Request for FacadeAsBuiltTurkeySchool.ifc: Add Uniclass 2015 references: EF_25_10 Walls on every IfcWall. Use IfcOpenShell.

First a look at what the model holds.

```python
import ifcopenshell

model = ifcopenshell.open("FacadeAsBuiltTurkeySchool.ifc")
print(model.schema)
print("classifications:", [c.Name for c in model.by_type("IfcClassification")])
for ifc_class in ("IfcDoor", "IfcRoof", "IfcStair", "IfcWall", "IfcWindow"):
    print(ifc_class, len(model.by_type(ifc_class)))
```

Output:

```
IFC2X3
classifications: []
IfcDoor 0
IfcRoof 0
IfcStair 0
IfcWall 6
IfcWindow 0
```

```python
import ifcopenshell
import ifcopenshell.api.classification

model = ifcopenshell.open("FacadeAsBuiltTurkeySchool.ifc")

# IFC2X3 requires Source and Edition and has no link from the project to the system.
system = model.create_entity("IfcClassification", Source="NBS", Edition="2015", Name="Uniclass 2015")

codes = {
    "IfcWall": ("EF_25_10", "Walls"),
}
for ifc_class, (code, name) in codes.items():
    products = model.by_type(ifc_class)
    ifcopenshell.api.classification.add_reference(
        model, products=products, classification=system, identification=code, name=name
    )
    print(code, len(products))

model.write("FacadeAsBuiltTurkeySchool-out.ifc")
```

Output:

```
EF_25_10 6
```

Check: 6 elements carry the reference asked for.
